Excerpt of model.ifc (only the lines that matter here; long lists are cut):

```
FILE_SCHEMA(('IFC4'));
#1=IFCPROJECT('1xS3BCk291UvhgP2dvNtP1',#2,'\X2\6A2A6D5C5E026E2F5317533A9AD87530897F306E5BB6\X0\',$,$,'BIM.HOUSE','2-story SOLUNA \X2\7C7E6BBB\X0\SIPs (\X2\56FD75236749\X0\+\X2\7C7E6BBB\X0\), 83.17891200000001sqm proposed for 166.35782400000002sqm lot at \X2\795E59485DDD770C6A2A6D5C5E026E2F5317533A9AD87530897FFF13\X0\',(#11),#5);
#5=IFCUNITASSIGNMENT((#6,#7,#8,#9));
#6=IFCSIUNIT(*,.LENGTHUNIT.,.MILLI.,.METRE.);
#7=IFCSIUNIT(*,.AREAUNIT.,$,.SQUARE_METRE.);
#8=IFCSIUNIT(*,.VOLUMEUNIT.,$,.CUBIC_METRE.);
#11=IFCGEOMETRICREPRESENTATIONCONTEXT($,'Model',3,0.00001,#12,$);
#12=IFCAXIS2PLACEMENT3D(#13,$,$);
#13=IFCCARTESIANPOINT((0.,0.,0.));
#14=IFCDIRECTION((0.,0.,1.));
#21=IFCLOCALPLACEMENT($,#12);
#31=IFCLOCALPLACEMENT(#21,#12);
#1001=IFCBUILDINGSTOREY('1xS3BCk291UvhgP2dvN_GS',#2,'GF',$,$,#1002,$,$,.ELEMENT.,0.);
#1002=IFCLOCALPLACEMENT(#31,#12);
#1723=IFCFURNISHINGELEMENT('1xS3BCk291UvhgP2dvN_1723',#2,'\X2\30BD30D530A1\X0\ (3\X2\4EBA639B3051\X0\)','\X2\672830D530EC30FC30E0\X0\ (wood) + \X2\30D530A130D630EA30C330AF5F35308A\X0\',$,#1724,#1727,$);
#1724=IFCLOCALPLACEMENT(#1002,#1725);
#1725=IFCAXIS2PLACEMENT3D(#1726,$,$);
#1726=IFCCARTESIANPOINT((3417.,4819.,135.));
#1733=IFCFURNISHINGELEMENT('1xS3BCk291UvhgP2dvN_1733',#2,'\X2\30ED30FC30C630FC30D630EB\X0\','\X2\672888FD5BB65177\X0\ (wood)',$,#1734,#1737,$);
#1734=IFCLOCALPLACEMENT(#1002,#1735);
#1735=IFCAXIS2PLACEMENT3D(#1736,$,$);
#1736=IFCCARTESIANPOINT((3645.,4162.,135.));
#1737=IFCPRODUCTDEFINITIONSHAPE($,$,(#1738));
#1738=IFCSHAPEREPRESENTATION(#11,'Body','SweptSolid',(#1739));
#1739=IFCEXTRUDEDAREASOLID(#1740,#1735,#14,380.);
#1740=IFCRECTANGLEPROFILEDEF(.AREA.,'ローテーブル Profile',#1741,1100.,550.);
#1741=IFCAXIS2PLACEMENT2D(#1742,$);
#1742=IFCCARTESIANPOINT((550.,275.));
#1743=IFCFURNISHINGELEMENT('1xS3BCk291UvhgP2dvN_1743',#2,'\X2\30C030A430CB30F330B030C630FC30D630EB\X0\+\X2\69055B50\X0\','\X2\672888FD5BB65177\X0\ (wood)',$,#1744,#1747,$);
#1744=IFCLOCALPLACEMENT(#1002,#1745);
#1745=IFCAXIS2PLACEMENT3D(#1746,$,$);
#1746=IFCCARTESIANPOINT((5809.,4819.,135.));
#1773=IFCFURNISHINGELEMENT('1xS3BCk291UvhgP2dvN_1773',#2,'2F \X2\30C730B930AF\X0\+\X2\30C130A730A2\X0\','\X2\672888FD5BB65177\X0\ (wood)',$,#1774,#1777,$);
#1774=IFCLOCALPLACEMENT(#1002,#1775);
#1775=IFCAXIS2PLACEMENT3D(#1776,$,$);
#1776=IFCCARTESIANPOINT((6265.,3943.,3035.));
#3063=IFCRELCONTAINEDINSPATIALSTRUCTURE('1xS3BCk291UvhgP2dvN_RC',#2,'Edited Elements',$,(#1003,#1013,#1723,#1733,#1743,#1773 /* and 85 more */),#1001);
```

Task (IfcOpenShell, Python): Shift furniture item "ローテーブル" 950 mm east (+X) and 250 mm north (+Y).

```python
import ifcopenshell
import ifcopenshell.api.geometry
import ifcopenshell.util.placement
import ifcopenshell.util.unit

model = ifcopenshell.open("model.ifc")
unit_scale = ifcopenshell.util.unit.calculate_unit_scale(model)

item = model.by_guid("1xS3BCk291UvhgP2dvN_1733")
matrix = ifcopenshell.util.placement.get_local_placement(item.ObjectPlacement)
matrix[0, 3] += 0.95 / unit_scale
matrix[1, 3] += 0.25 / unit_scale
ifcopenshell.api.geometry.edit_object_placement(model, product=item, matrix=matrix, is_si=False)

print(ifcopenshell.util.placement.get_local_placement(item.ObjectPlacement).round(3) + 0.0)

model.write("model_v2.ifc")
```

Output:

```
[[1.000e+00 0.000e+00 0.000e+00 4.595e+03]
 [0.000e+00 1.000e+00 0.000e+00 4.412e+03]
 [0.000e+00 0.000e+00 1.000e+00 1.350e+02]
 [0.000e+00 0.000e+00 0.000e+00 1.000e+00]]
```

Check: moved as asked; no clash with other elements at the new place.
